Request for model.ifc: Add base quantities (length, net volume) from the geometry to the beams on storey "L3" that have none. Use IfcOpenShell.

First a look at what the model holds.

```python
import ifcopenshell
import ifcopenshell.util.element
import ifcopenshell.util.unit

model = ifcopenshell.open("model.ifc")
print(model.schema)
for unit_type in ("LENGTHUNIT", "AREAUNIT", "VOLUMEUNIT"):
    print(unit_type, ifcopenshell.util.unit.calculate_unit_scale(model, unit_type))
storey = next(s for s in model.by_type("IfcBuildingStorey") if s.Name == "L3")
beams = [e for e in ifcopenshell.util.element.get_decomposition(storey) if e.is_a("IfcBeam")]
for e in sorted(beams, key=lambda e: e.id()):
    print(e.id(), e.is_a(), e.Name, list(ifcopenshell.util.element.get_psets(e, qtos_only=True)), sep=" | ")
```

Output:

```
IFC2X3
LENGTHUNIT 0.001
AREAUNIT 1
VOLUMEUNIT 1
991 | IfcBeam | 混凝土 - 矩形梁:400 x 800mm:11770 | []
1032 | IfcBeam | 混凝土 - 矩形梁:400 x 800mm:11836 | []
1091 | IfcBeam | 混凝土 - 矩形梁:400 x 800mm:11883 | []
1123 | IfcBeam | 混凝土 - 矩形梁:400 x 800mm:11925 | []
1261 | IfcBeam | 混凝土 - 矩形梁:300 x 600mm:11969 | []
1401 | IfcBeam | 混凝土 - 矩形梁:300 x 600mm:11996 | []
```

```python
import ifcopenshell
import ifcopenshell.api.pset
import ifcopenshell.geom
import ifcopenshell.util.element
import ifcopenshell.util.shape
import ifcopenshell.util.unit

model = ifcopenshell.open("model.ifc")
unit_scale = ifcopenshell.util.unit.calculate_unit_scale(model)
volume_scale = ifcopenshell.util.unit.calculate_unit_scale(model, "VOLUMEUNIT")
settings = ifcopenshell.geom.settings()

storey = next(s for s in model.by_type("IfcBuildingStorey") if s.Name == "L3")
beams = [e for e in ifcopenshell.util.element.get_decomposition(storey) if e.is_a("IfcBeam")]

for e in sorted(beams, key=lambda e: e.id()):
    if ifcopenshell.util.element.get_psets(e, qtos_only=True, should_inherit=False):
        continue
    # Geometry comes back in metres, in the element's own axes.
    shape = ifcopenshell.geom.create_shape(settings, e)
    values = {
        "Length": ifcopenshell.util.shape.get_max_xyz(shape.geometry) / unit_scale,
        "NetVolume": ifcopenshell.util.shape.get_volume(shape.geometry) / volume_scale,
    }
    qto = ifcopenshell.api.pset.add_qto(model, product=e, name="BaseQuantities")
    ifcopenshell.api.pset.edit_qto(model, qto=qto, properties=values)
    print(e.id(), {k: round(v, 3) for k, v in values.items()})

model.write("model_updated.ifc")
```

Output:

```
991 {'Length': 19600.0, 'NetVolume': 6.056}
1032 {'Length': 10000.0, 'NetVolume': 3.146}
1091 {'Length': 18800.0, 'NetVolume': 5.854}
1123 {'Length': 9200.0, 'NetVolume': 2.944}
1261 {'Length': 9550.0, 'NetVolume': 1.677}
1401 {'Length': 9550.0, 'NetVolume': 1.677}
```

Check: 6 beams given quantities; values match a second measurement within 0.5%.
